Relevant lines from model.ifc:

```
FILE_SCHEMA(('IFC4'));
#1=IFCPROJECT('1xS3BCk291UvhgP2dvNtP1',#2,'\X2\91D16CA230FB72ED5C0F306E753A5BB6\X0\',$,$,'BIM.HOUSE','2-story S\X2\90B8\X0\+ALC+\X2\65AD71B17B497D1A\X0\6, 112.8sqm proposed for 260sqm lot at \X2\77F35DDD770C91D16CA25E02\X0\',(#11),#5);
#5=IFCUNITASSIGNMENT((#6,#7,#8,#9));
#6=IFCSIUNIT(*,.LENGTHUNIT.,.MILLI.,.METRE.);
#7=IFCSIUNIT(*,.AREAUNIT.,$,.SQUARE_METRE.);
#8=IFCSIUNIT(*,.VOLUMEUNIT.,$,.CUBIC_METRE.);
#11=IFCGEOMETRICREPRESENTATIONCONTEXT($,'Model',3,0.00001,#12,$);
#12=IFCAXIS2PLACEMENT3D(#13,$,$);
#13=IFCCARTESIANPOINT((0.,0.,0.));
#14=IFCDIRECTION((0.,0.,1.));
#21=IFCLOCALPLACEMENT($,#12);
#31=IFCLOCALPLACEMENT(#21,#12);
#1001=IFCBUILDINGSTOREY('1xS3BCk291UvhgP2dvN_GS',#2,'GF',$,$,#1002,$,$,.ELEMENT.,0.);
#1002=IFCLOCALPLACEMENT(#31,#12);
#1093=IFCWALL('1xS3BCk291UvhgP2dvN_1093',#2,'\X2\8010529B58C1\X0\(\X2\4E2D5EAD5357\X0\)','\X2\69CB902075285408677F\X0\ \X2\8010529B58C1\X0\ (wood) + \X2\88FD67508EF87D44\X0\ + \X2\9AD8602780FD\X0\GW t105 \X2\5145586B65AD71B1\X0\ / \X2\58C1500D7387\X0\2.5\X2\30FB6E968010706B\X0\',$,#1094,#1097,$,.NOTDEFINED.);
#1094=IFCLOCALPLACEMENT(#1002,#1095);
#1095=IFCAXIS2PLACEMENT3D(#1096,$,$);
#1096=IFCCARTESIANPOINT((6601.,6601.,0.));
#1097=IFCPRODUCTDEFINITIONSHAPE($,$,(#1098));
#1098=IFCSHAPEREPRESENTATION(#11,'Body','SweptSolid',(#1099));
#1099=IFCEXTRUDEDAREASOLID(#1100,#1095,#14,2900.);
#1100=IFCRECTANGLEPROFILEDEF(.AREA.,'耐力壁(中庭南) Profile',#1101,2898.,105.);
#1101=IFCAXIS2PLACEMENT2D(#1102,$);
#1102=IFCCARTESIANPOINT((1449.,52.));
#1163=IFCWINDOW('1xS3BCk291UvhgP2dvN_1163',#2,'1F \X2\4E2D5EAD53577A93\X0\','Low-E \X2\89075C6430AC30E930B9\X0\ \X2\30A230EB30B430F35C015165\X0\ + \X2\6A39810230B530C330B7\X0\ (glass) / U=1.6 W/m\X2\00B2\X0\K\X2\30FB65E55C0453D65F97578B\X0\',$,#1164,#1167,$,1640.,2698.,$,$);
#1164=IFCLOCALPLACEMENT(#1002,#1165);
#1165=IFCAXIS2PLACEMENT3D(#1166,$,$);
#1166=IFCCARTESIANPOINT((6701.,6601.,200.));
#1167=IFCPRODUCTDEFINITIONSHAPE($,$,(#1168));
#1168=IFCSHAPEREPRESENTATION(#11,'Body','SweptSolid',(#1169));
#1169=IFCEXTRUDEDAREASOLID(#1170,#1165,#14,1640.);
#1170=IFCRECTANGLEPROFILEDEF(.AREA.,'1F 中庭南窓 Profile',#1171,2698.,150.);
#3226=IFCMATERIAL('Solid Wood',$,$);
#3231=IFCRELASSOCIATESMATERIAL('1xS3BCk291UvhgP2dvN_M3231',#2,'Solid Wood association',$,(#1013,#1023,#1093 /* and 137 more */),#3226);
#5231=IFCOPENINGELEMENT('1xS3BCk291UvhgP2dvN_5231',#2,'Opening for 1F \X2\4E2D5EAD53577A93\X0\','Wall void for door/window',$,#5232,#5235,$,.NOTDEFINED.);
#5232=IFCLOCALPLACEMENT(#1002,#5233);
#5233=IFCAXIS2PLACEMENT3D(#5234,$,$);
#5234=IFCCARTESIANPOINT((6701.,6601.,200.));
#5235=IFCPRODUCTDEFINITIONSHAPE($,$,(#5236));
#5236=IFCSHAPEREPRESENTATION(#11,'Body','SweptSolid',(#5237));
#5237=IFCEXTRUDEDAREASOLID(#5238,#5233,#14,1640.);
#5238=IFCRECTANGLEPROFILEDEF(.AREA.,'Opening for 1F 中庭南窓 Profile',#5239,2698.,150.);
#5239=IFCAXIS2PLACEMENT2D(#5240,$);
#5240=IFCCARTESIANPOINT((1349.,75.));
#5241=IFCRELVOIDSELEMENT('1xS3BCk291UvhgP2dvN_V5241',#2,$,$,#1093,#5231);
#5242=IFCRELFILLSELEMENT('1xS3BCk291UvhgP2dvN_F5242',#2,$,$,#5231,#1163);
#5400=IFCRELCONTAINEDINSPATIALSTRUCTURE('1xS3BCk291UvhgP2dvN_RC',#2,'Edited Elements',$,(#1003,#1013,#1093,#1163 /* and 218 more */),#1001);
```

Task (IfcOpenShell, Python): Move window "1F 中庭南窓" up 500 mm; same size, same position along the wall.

```python
import numpy as np
import ifcopenshell
import ifcopenshell.api.geometry
import ifcopenshell.util.placement
import ifcopenshell.util.unit

model = ifcopenshell.open("model.ifc")
unit_scale = ifcopenshell.util.unit.calculate_unit_scale(model)

window = model.by_guid("1xS3BCk291UvhgP2dvN_1163")
opening = window.FillsVoids[0].RelatingOpeningElement
dz = 500.0

shift = np.array([0.0, 0.0, dz])
# The window is not placed relative to its opening, so move both.
for product in (opening, window):
    matrix = ifcopenshell.util.placement.get_local_placement(product.ObjectPlacement)
    matrix[:3, 3] += shift
    ifcopenshell.api.geometry.edit_object_placement(model, product=product, matrix=matrix, is_si=False)

print(f"moved by {dz * unit_scale:+.3f} m")

model.write("model_edited.ifc")
```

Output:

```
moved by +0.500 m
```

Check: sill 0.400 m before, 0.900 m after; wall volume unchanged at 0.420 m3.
